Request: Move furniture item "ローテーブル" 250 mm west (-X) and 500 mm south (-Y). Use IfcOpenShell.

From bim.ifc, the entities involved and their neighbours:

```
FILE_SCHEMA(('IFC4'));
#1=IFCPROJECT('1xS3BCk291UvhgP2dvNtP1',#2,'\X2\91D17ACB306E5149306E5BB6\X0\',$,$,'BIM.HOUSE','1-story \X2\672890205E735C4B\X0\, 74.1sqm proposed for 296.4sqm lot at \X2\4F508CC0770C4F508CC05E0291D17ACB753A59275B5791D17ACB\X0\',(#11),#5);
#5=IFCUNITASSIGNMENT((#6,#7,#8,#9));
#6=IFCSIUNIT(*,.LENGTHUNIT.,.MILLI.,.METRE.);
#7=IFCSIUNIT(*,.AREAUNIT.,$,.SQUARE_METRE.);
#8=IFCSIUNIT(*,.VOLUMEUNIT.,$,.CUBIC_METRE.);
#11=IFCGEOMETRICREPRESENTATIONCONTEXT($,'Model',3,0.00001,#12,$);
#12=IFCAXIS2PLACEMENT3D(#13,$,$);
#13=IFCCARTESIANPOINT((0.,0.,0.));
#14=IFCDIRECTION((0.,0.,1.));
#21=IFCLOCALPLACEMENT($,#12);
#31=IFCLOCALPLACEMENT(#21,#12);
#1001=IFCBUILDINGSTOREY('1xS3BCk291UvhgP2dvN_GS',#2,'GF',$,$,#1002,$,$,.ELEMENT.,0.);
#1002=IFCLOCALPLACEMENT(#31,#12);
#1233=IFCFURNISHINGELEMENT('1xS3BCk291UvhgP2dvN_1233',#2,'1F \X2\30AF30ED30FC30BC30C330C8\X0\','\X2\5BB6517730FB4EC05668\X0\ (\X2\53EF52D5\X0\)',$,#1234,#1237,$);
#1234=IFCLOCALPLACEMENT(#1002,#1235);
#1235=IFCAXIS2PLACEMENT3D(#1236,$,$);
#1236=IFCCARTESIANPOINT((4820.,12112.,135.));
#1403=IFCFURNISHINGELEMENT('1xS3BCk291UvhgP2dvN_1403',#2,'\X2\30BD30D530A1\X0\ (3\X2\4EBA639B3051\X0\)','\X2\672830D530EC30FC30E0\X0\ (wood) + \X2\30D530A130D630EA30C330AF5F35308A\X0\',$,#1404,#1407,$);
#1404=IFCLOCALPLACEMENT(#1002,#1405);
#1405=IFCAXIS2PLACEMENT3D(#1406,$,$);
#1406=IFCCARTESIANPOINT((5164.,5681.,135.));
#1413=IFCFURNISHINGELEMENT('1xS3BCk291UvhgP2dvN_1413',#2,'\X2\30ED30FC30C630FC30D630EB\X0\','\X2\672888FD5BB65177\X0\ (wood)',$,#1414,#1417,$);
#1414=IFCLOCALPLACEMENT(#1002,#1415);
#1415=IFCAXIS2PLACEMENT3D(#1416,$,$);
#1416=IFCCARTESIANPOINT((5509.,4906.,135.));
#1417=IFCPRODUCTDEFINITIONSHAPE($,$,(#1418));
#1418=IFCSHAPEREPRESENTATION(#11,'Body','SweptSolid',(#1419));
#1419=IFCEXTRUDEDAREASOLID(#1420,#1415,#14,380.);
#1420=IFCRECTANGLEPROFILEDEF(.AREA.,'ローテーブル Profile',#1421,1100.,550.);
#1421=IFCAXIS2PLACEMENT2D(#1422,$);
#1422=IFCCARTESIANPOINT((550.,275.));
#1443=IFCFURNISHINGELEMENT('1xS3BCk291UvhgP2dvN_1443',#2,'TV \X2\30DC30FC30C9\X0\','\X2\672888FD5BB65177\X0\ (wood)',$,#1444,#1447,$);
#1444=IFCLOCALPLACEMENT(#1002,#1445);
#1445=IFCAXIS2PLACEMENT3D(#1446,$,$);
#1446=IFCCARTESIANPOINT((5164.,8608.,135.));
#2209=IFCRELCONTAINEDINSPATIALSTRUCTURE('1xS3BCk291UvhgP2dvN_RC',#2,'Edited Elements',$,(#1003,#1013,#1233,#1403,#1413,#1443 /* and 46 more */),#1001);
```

```python
import ifcopenshell
import ifcopenshell.api.geometry
import ifcopenshell.util.placement
import ifcopenshell.util.unit

model = ifcopenshell.open("bim.ifc")
unit_scale = ifcopenshell.util.unit.calculate_unit_scale(model)

item = model.by_id(1413)
matrix = ifcopenshell.util.placement.get_local_placement(item.ObjectPlacement)
matrix[0, 3] -= 0.25 / unit_scale
matrix[1, 3] -= 0.5 / unit_scale
ifcopenshell.api.geometry.edit_object_placement(model, product=item, matrix=matrix, is_si=False)

print(ifcopenshell.util.placement.get_local_placement(item.ObjectPlacement).round(3) + 0.0)

model.write("bim_edited.ifc")
```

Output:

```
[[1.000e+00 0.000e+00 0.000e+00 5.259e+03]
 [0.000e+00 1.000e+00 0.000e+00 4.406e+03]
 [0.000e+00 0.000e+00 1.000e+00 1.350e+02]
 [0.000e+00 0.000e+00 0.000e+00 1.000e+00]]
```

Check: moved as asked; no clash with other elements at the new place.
